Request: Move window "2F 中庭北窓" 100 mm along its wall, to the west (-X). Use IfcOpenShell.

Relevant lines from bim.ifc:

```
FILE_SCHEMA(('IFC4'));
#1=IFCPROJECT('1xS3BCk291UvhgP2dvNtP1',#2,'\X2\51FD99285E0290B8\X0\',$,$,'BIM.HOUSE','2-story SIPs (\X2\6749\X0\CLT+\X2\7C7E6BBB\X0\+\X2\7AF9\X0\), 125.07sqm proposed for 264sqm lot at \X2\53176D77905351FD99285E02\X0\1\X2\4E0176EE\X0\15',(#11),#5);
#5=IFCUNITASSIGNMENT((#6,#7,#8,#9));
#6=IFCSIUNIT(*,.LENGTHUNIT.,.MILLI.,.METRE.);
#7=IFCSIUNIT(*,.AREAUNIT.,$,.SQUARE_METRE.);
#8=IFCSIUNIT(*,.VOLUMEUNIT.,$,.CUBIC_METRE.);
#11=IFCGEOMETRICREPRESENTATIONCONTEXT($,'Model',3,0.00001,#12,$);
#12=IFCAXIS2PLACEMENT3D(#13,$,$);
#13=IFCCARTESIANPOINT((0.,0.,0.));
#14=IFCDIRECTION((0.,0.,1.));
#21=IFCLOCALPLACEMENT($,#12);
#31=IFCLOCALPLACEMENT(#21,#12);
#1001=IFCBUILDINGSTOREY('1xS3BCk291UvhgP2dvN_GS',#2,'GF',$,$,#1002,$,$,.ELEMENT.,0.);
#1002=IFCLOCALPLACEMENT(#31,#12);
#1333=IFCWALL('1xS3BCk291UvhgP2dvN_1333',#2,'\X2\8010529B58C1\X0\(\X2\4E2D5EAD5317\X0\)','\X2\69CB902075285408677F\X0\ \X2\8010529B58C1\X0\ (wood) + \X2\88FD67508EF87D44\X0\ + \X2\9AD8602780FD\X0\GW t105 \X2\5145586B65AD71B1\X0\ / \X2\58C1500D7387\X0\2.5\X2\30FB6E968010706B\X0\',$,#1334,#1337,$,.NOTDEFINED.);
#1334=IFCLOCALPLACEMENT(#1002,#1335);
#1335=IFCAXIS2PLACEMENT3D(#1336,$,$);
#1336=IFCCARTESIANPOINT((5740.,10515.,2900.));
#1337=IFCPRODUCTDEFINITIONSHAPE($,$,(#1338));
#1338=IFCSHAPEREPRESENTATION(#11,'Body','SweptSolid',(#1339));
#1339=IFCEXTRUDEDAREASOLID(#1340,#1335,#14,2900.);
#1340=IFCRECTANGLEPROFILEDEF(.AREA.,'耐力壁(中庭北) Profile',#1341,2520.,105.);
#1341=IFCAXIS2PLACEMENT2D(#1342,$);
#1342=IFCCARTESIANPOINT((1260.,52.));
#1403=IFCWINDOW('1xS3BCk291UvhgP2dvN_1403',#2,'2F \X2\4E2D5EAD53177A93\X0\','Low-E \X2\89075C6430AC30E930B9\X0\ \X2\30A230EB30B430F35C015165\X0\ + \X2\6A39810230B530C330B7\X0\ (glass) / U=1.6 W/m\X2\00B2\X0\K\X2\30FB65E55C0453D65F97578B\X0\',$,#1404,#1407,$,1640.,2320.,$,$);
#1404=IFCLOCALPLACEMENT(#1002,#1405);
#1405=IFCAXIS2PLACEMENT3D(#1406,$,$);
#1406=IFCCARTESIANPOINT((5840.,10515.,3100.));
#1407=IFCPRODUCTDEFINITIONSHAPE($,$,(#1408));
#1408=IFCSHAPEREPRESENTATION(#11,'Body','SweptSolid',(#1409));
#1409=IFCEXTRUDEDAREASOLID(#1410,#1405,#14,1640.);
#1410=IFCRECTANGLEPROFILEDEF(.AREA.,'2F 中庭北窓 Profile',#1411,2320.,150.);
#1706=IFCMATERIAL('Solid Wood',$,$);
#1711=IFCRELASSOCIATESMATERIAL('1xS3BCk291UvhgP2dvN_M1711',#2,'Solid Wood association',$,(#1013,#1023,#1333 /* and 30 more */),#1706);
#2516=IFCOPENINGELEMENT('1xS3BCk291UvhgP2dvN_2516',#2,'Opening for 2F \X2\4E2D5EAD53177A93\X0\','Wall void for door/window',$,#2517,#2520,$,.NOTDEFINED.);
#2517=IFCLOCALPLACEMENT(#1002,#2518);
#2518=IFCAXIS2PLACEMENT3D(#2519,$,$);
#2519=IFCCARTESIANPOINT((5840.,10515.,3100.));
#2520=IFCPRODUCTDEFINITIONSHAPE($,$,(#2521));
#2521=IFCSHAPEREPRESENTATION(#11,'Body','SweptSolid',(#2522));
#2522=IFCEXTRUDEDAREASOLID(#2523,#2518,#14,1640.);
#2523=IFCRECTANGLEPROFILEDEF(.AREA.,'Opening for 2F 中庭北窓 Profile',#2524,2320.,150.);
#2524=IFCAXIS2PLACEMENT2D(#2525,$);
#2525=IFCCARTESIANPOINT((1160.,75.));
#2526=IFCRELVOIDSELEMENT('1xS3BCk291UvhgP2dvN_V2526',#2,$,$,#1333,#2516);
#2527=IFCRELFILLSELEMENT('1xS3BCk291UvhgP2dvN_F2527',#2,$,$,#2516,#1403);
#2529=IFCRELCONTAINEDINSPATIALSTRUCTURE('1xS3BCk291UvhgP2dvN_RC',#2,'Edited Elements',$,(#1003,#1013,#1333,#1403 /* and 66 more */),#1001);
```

```python
import ifcopenshell
import ifcopenshell.api.geometry
import ifcopenshell.util.placement
import ifcopenshell.util.unit

model = ifcopenshell.open("bim.ifc")
unit_scale = ifcopenshell.util.unit.calculate_unit_scale(model)

window = model.by_guid("1xS3BCk291UvhgP2dvN_1403")
opening = window.FillsVoids[0].RelatingOpeningElement
wall = opening.VoidsElements[0].RelatingBuildingElement

wall_matrix = ifcopenshell.util.placement.get_local_placement(wall.ObjectPlacement)
shift = wall_matrix[:3, 0] * -0.1 / unit_scale
before = ifcopenshell.util.placement.get_local_placement(window.ObjectPlacement)[:3, 3].copy()

# The window is not placed relative to its opening, so move both.
for product in (opening, window):
    matrix = ifcopenshell.util.placement.get_local_placement(product.ObjectPlacement)
    matrix[:3, 3] += shift
    ifcopenshell.api.geometry.edit_object_placement(model, product=product, matrix=matrix, is_si=False)

after = ifcopenshell.util.placement.get_local_placement(window.ObjectPlacement)[:3, 3]
print("window moved by", (after - before).round(3) + 0.0)

model.write("bim_edited.ifc")
```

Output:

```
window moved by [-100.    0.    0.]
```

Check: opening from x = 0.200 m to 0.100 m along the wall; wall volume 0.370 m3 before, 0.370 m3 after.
